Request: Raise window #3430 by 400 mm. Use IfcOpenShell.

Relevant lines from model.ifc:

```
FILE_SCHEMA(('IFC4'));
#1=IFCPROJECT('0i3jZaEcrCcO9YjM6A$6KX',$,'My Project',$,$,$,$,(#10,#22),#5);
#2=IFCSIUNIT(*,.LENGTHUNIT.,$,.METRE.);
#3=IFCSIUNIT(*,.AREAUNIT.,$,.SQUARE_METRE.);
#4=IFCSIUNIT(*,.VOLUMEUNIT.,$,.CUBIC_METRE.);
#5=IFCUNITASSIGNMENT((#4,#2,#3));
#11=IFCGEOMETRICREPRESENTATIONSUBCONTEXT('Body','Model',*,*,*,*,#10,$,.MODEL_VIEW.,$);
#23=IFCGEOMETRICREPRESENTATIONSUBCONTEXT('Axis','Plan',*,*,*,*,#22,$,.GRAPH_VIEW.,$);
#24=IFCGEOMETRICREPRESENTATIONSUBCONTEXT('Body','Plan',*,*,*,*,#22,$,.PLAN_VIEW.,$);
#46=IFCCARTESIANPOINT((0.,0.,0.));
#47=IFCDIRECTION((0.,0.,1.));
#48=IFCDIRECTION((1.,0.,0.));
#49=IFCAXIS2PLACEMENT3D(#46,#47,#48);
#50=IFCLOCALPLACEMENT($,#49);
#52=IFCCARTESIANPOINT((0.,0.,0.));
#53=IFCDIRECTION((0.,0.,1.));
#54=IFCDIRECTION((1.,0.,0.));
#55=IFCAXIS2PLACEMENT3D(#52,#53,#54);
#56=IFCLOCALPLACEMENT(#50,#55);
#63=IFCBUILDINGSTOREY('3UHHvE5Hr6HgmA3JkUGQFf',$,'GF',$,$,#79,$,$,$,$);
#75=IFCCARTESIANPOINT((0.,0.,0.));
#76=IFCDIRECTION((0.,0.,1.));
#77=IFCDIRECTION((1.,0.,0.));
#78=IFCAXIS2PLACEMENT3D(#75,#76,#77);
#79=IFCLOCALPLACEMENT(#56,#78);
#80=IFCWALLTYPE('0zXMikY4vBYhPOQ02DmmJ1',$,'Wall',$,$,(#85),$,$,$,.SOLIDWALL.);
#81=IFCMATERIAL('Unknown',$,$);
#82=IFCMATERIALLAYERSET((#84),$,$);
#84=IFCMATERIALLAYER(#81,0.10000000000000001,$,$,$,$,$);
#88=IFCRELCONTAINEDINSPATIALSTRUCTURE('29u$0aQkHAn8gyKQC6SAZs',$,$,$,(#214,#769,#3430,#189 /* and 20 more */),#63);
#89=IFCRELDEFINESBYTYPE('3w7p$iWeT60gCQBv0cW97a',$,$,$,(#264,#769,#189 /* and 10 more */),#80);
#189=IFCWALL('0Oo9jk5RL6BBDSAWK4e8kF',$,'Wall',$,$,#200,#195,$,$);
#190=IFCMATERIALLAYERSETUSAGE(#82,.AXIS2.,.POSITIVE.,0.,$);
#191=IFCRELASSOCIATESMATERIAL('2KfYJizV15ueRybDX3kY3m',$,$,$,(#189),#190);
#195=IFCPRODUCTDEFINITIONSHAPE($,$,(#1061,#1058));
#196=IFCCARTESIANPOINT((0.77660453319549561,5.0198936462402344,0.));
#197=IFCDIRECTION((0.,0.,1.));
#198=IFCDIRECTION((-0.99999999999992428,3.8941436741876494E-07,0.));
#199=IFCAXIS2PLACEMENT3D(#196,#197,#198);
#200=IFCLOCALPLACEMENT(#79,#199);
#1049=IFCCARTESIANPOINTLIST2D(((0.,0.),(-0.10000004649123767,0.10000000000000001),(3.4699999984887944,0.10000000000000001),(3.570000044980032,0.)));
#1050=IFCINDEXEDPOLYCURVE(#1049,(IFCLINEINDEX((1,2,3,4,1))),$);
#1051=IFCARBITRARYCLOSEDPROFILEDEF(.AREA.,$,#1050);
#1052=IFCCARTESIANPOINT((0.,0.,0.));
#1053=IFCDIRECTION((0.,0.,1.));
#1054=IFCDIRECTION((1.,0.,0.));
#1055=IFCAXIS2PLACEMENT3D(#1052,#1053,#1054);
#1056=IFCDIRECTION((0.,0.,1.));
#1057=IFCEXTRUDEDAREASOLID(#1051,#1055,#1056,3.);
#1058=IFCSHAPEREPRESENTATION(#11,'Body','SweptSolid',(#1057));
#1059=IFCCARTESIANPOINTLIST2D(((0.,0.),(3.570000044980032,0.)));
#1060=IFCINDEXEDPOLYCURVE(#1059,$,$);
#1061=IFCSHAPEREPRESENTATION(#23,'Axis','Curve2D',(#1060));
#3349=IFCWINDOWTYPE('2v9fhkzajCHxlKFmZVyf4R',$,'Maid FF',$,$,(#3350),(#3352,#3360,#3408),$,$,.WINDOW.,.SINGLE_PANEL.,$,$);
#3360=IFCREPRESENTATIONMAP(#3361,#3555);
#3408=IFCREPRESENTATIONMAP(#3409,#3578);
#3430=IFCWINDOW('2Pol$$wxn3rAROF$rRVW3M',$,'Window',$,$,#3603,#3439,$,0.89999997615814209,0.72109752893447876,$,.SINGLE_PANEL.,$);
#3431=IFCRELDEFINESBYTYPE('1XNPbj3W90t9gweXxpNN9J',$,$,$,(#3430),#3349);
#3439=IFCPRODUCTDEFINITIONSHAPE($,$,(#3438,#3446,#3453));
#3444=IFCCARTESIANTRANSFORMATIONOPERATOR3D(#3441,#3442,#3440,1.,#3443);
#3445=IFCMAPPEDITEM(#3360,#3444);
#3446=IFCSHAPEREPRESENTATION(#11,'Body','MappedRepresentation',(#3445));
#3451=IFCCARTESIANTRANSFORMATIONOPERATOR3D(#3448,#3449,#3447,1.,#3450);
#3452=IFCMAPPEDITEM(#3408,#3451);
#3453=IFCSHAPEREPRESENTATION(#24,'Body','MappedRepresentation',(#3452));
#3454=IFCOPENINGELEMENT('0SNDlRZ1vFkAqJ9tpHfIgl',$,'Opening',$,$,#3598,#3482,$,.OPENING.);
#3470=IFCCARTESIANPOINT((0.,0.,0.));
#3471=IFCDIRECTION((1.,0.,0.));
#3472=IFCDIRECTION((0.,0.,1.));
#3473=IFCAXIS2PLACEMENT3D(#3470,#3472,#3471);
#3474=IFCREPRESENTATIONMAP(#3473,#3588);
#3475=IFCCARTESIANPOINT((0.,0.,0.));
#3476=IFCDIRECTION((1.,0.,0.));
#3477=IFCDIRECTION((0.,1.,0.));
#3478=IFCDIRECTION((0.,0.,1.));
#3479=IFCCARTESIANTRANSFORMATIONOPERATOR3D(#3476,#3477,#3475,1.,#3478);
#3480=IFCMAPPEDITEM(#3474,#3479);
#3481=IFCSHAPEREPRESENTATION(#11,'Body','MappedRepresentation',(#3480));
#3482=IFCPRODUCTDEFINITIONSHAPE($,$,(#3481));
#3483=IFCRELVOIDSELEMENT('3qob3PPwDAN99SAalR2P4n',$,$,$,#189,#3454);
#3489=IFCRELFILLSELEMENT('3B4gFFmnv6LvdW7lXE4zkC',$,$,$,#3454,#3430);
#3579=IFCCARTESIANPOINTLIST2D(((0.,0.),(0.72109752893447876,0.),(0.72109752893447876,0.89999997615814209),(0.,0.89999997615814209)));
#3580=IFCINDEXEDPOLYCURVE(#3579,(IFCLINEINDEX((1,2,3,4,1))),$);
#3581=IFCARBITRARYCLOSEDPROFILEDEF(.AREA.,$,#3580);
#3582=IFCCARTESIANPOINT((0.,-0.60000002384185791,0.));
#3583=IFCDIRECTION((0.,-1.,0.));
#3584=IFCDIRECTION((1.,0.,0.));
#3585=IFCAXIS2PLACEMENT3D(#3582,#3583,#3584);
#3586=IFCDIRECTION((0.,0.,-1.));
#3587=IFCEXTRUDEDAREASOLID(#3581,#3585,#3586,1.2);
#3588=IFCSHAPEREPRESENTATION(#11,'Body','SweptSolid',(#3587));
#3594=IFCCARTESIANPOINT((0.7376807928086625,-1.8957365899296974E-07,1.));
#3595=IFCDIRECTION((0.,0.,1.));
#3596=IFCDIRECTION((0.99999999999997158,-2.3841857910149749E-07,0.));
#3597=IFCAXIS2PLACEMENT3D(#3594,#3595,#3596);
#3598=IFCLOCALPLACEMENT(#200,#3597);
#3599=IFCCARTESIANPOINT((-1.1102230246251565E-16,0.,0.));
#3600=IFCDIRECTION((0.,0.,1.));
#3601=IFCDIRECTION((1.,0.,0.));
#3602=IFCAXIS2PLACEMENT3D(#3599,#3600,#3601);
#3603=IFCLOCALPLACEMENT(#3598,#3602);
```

```python
import numpy as np
import ifcopenshell
import ifcopenshell.api.geometry
import ifcopenshell.util.placement
import ifcopenshell.util.unit

model = ifcopenshell.open("model.ifc")
unit_scale = ifcopenshell.util.unit.calculate_unit_scale(model)

window = model.by_guid("2Pol$$wxn3rAROF$rRVW3M")
opening = window.FillsVoids[0].RelatingOpeningElement
dz = 0.4

shift = np.array([0.0, 0.0, dz])
# The window is placed relative to its opening, so it follows when the opening moves.
matrix = ifcopenshell.util.placement.get_local_placement(opening.ObjectPlacement)
matrix[:3, 3] += shift
ifcopenshell.api.geometry.edit_object_placement(
    model, product=opening, matrix=matrix, is_si=False, should_transform_children=True
)

print(f"moved by {dz * unit_scale:+.3f} m")

model.write("model-out.ifc")
```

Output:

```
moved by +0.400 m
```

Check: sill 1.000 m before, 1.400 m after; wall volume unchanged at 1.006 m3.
